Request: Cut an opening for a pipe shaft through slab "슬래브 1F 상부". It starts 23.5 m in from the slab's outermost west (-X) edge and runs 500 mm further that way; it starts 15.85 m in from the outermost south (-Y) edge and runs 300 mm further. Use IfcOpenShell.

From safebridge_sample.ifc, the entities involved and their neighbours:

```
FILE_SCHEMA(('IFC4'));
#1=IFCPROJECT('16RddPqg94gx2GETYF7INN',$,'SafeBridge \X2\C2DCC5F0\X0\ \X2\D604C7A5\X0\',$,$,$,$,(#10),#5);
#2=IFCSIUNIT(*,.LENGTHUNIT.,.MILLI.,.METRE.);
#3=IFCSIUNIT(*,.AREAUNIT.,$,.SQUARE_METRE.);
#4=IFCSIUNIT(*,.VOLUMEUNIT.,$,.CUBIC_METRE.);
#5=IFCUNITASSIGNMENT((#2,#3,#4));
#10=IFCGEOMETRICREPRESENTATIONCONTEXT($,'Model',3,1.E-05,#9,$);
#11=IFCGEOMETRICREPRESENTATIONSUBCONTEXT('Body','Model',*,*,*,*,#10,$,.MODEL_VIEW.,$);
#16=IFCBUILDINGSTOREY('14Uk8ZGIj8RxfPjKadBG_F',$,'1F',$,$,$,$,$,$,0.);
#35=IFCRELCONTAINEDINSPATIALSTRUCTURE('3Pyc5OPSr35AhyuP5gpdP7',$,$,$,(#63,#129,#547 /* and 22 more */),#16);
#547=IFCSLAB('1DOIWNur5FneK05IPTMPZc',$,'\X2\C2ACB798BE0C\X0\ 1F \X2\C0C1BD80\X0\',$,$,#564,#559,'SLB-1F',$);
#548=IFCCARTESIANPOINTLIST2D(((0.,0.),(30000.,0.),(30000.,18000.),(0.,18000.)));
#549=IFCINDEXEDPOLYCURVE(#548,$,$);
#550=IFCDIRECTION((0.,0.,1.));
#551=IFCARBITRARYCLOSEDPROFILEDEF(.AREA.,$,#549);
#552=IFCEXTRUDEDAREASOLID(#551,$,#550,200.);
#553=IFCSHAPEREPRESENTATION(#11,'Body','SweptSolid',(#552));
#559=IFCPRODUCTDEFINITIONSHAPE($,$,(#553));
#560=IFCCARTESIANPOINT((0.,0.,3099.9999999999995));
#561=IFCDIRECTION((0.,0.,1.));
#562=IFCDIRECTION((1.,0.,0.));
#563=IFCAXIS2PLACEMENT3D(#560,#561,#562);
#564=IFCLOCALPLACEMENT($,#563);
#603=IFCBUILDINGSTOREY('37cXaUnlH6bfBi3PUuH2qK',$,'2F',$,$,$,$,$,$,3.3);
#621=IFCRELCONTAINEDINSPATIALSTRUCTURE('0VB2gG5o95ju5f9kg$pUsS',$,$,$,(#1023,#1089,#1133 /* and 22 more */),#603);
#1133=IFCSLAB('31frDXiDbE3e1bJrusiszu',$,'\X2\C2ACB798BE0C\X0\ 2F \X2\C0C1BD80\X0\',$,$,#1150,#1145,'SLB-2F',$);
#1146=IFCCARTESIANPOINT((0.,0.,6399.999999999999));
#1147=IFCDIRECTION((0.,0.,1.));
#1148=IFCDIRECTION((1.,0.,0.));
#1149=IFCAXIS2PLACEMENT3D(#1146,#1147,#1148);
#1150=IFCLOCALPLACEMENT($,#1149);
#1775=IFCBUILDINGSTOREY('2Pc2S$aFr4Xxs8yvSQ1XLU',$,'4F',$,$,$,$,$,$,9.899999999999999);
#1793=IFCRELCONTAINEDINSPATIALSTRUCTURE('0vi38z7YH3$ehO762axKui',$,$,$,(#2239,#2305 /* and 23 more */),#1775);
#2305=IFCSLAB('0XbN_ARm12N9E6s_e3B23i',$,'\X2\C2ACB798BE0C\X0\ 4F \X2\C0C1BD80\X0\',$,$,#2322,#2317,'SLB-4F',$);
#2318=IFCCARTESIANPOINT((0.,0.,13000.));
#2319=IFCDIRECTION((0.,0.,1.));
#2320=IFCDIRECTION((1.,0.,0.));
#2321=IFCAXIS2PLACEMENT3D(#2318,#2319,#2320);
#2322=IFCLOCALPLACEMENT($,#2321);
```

```python
import numpy as np
import ifcopenshell
import ifcopenshell.api.feature
import ifcopenshell.api.geometry
import ifcopenshell.api.root
import ifcopenshell.geom
import ifcopenshell.util.placement
import ifcopenshell.util.representation
import ifcopenshell.util.shape
import ifcopenshell.util.unit

model = ifcopenshell.open("safebridge_sample.ifc")
unit_scale = ifcopenshell.util.unit.calculate_unit_scale(model)
settings = ifcopenshell.geom.settings()


def volume(element):
    """Net volume in cubic metres, openings subtracted."""
    shape = ifcopenshell.geom.create_shape(settings, element)
    return ifcopenshell.util.shape.get_volume(shape.geometry)


slab = model.by_guid("1DOIWNur5FneK05IPTMPZc")
before = volume(slab)

# Extent in the slab's own axes, in metres. The edges named are its -X and -Y sides.
slab_shape = ifcopenshell.geom.create_shape(settings, slab)
vertices = ifcopenshell.util.shape.get_vertices(slab_shape.geometry)
x_min, y_min, bottom = vertices.min(axis=0)
top = vertices[:, 2].max()

opening = ifcopenshell.api.root.create_entity(model, ifc_class="IfcOpeningElement", name="Pipe shaft opening", predefined_type="OPENING")
context = ifcopenshell.util.representation.get_context(model, "Model", "Body", "MODEL_VIEW")
width, depth = 0.5, 0.3
outline = [(0.0, 0.0), (width, 0.0), (width, depth), (0.0, depth), (0.0, 0.0)]
# Overshoot both faces by 50 mm so the cut is clean.
shape = ifcopenshell.api.geometry.add_slab_representation(
    model, context=context, depth=top - bottom + 0.1, polyline=outline
)
ifcopenshell.api.geometry.assign_representation(model, product=opening, representation=shape)

matrix = ifcopenshell.util.placement.get_local_placement(slab.ObjectPlacement)
matrix[:, 3] = matrix @ np.append(np.array([x_min + 23.5, y_min + 15.85, bottom - 0.05]) / unit_scale, 1.0)
ifcopenshell.api.geometry.edit_object_placement(model, product=opening, matrix=matrix, is_si=False)
ifcopenshell.api.feature.add_feature(model, feature=opening, element=slab)

after = volume(slab)

print(f"slab volume {before:.3f} -> {after:.3f} m3")

model.write("safebridge_sample-out.ifc")
```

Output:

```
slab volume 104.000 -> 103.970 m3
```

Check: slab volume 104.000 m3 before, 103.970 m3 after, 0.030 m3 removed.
